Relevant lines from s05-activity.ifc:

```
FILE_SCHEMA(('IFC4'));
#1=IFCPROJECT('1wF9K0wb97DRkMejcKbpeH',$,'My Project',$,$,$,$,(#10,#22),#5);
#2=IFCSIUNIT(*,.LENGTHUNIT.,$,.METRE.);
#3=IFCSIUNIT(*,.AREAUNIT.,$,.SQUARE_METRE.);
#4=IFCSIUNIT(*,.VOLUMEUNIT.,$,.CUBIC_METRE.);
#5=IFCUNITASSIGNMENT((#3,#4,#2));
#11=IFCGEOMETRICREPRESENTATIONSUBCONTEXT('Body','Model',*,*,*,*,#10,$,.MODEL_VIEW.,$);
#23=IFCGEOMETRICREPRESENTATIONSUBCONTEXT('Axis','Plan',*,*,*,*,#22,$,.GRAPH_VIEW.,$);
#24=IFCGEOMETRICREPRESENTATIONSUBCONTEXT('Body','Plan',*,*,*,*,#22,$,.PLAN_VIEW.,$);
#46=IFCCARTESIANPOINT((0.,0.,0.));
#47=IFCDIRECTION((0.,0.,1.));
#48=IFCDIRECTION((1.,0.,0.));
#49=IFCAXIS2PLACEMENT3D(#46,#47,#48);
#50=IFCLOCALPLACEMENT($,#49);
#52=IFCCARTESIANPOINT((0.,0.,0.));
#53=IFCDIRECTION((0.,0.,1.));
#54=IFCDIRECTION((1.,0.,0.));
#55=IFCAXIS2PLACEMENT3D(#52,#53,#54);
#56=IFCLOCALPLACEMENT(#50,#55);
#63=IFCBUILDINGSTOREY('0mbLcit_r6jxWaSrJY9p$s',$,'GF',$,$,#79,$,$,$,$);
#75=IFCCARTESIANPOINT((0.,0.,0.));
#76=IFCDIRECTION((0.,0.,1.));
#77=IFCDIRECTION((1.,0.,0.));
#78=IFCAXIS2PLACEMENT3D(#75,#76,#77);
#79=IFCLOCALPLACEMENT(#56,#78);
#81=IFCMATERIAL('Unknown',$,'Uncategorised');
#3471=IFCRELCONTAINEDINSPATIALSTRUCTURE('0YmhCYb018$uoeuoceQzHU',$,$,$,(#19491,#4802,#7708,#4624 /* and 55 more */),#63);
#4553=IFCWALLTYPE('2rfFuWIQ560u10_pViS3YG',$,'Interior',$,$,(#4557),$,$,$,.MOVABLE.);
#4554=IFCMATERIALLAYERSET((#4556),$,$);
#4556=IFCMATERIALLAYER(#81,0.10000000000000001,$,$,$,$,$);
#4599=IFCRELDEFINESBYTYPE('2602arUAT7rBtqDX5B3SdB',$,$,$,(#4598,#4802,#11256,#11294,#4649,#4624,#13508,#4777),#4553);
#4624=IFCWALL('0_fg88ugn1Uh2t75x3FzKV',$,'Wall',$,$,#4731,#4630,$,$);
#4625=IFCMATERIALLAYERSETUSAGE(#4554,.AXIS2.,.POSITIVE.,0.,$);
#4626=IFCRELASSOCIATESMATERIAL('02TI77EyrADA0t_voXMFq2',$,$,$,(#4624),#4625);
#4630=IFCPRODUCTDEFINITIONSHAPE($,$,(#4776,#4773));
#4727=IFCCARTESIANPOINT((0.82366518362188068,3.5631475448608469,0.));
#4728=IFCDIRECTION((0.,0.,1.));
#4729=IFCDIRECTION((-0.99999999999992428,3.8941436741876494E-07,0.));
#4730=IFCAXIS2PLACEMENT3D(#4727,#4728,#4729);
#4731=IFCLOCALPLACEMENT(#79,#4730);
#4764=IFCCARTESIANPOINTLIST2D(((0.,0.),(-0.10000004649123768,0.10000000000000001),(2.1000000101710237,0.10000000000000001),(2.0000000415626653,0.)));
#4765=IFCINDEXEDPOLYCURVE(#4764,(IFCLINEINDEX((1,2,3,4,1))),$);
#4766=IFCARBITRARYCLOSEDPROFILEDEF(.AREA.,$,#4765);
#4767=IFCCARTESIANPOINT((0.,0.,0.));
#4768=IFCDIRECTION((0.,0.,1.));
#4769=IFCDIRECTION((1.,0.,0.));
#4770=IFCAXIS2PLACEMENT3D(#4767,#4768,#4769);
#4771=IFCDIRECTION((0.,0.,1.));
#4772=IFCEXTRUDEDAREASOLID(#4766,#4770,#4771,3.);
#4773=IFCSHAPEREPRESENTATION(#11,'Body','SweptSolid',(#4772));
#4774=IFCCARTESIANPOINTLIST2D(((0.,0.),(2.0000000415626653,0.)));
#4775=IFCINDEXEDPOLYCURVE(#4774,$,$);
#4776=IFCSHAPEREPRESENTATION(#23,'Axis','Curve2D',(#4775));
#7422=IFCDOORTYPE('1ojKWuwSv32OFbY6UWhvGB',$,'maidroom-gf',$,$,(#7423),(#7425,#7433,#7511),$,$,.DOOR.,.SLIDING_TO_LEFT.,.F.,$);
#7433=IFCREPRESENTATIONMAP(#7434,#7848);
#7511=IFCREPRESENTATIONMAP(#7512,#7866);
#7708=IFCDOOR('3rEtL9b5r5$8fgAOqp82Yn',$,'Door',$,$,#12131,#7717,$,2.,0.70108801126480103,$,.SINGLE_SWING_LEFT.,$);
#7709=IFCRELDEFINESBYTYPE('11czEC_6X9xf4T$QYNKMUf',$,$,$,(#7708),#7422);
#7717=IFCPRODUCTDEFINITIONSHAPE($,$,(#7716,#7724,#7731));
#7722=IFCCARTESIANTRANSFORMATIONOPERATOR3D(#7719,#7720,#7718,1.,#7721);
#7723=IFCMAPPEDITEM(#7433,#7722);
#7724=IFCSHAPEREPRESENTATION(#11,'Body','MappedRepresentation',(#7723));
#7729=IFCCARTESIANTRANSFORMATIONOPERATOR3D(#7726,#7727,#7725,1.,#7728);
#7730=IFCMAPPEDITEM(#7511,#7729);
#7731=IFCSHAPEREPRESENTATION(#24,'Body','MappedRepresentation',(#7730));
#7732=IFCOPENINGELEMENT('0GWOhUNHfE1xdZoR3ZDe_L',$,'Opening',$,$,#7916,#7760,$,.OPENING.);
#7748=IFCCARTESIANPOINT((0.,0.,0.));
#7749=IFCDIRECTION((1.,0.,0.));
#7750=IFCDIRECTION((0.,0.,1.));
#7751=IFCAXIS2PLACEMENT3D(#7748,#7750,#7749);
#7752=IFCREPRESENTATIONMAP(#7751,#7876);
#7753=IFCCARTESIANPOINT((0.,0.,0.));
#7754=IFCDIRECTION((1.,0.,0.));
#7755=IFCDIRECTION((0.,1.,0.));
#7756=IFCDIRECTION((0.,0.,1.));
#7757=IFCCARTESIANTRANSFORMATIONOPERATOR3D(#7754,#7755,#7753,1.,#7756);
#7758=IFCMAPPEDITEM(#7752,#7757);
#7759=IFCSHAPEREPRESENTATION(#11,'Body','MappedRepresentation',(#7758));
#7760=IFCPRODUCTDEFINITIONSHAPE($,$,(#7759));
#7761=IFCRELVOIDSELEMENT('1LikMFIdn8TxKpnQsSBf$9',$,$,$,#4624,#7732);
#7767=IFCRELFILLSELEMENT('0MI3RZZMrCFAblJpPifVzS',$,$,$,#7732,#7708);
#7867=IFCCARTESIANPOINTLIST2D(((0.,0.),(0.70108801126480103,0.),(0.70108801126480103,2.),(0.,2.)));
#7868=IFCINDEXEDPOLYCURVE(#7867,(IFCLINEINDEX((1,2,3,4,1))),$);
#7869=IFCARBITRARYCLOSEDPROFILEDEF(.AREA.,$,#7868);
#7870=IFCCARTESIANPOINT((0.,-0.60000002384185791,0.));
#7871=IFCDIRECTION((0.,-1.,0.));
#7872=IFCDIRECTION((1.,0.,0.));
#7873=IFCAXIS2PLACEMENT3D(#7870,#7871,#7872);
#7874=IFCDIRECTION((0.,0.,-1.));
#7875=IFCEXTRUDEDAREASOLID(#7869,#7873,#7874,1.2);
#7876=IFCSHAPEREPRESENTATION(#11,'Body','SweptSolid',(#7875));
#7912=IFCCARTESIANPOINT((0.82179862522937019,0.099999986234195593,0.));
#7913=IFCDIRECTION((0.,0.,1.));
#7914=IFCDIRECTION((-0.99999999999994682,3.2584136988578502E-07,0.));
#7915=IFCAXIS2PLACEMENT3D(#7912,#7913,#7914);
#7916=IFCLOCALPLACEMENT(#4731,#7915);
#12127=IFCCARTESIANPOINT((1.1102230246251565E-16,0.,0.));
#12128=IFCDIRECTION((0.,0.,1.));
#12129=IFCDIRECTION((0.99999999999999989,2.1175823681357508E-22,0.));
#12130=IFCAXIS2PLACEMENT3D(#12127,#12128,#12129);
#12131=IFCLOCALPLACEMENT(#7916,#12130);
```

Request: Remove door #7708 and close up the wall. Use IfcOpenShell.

```python
import ifcopenshell
import ifcopenshell.api.feature
import ifcopenshell.api.root
import ifcopenshell.geom
import ifcopenshell.util.shape

model = ifcopenshell.open("s05-activity.ifc")
settings = ifcopenshell.geom.settings()


def volume(element):
    """Net volume in cubic metres, openings subtracted."""
    shape = ifcopenshell.geom.create_shape(settings, element)
    return ifcopenshell.util.shape.get_volume(shape.geometry)


door = model.by_guid("3rEtL9b5r5$8fgAOqp82Yn")
opening = door.FillsVoids[0].RelatingOpeningElement
wall = opening.VoidsElements[0].RelatingBuildingElement
before = volume(wall)

ifcopenshell.api.root.remove_product(model, product=door)
ifcopenshell.api.feature.remove_feature(model, feature=opening)

after = volume(wall)

print(f"wall volume {before:.3f} -> {after:.3f} m3")

model.write("s05-activity_v2.ifc")
```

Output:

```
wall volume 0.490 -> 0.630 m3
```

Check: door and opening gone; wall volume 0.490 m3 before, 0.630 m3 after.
